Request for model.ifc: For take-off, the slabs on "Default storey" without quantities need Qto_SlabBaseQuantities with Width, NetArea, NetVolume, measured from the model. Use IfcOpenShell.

First a look at what the model holds.

```python
import ifcopenshell
import ifcopenshell.util.element
import ifcopenshell.util.unit

model = ifcopenshell.open("model.ifc")
print(model.schema)
for unit_type in ("LENGTHUNIT", "AREAUNIT", "VOLUMEUNIT"):
    print(unit_type, ifcopenshell.util.unit.calculate_unit_scale(model, unit_type))
storey = next(s for s in model.by_type("IfcBuildingStorey") if s.Name == "Default storey")
slabs = [e for e in ifcopenshell.util.element.get_decomposition(storey) if e.is_a("IfcSlab")]
for e in sorted(slabs, key=lambda e: e.id()):
    print(e.id(), e.is_a(), e.Name, list(ifcopenshell.util.element.get_psets(e, qtos_only=True)), sep=" | ")
```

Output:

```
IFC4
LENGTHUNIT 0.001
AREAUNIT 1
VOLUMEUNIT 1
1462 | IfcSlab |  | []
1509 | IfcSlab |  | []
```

```python
import ifcopenshell
import ifcopenshell.api.pset
import ifcopenshell.geom
import ifcopenshell.util.element
import ifcopenshell.util.shape
import ifcopenshell.util.unit

model = ifcopenshell.open("model.ifc")
unit_scale = ifcopenshell.util.unit.calculate_unit_scale(model)
area_scale = ifcopenshell.util.unit.calculate_unit_scale(model, "AREAUNIT")
volume_scale = ifcopenshell.util.unit.calculate_unit_scale(model, "VOLUMEUNIT")
settings = ifcopenshell.geom.settings()

storey = next(s for s in model.by_type("IfcBuildingStorey") if s.Name == "Default storey")
slabs = [e for e in ifcopenshell.util.element.get_decomposition(storey) if e.is_a("IfcSlab")]

for e in sorted(slabs, key=lambda e: e.id()):
    if ifcopenshell.util.element.get_psets(e, qtos_only=True, should_inherit=False):
        continue
    # Geometry comes back in metres, in the element's own axes.
    shape = ifcopenshell.geom.create_shape(settings, e)
    values = {
        "Width": ifcopenshell.util.shape.get_z(shape.geometry) / unit_scale,
        "NetArea": ifcopenshell.util.shape.get_footprint_area(shape.geometry) / area_scale,
        "NetVolume": ifcopenshell.util.shape.get_volume(shape.geometry) / volume_scale,
    }
    qto = ifcopenshell.api.pset.add_qto(model, product=e, name="Qto_SlabBaseQuantities")
    ifcopenshell.api.pset.edit_qto(model, qto=qto, properties=values)
    print(e.id(), {k: round(v, 3) for k, v in values.items()})

model.write("model-out.ifc")
```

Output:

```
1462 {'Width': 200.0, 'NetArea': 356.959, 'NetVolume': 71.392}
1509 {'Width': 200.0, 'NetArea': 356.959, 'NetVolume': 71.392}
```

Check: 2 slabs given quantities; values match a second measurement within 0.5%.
